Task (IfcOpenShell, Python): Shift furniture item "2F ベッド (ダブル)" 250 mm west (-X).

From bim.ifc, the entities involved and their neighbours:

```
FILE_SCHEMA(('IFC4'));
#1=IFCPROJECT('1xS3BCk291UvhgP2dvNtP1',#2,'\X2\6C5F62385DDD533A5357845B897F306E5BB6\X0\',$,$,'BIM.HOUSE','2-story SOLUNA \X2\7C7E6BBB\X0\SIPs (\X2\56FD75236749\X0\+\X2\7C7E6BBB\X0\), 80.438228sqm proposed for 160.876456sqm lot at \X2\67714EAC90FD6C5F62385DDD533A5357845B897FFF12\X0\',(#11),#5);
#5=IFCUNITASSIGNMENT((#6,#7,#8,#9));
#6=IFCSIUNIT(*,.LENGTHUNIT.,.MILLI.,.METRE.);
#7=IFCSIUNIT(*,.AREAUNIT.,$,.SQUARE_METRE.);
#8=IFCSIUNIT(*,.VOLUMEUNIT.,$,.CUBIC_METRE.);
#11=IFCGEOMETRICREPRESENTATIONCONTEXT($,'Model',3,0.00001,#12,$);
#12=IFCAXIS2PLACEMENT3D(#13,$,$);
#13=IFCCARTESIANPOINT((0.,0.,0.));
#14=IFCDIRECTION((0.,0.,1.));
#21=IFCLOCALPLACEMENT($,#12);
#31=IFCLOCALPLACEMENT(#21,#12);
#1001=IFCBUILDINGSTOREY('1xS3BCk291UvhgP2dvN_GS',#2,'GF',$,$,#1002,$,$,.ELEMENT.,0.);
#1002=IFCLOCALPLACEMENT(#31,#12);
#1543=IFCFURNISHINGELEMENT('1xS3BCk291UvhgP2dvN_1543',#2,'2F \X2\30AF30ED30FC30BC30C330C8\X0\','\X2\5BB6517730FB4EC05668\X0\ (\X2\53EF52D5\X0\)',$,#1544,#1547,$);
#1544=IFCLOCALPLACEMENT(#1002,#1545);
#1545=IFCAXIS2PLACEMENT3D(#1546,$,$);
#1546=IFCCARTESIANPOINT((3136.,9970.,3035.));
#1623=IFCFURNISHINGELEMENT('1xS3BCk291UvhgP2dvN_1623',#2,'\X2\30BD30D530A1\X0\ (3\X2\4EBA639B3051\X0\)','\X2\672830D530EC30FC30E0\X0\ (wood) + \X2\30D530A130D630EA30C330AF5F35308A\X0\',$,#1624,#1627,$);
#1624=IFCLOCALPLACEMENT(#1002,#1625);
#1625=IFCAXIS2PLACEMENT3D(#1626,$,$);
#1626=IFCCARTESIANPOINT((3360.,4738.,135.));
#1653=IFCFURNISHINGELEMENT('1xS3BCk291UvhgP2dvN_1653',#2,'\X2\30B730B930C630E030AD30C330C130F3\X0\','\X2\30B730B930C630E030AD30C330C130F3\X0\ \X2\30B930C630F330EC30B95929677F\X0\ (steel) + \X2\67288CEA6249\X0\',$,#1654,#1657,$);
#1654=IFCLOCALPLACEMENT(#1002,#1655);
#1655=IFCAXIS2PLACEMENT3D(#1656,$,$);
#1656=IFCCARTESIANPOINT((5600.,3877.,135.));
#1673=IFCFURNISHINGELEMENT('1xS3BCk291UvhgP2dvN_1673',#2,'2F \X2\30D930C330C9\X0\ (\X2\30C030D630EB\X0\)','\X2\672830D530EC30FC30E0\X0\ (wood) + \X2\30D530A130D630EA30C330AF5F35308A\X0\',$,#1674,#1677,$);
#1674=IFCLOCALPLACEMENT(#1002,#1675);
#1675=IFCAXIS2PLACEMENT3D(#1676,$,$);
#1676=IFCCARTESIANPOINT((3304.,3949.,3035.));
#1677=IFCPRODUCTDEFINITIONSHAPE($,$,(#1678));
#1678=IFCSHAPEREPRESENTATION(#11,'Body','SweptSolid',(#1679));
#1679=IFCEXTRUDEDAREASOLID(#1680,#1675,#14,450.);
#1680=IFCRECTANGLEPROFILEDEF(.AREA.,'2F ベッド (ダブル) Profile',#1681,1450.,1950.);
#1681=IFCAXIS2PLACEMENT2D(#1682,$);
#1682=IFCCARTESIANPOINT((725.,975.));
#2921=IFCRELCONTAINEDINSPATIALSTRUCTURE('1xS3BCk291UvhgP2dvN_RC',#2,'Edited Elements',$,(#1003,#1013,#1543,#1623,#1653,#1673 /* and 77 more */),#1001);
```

```python
import ifcopenshell
import ifcopenshell.api.geometry
import ifcopenshell.util.placement
import ifcopenshell.util.unit

model = ifcopenshell.open("bim.ifc")
unit_scale = ifcopenshell.util.unit.calculate_unit_scale(model)

item = model.by_guid("1xS3BCk291UvhgP2dvN_1673")
matrix = ifcopenshell.util.placement.get_local_placement(item.ObjectPlacement)
matrix[0, 3] -= 0.25 / unit_scale
ifcopenshell.api.geometry.edit_object_placement(model, product=item, matrix=matrix, is_si=False)

print(ifcopenshell.util.placement.get_local_placement(item.ObjectPlacement).round(3) + 0.0)

model.write("bim_v2.ifc")
```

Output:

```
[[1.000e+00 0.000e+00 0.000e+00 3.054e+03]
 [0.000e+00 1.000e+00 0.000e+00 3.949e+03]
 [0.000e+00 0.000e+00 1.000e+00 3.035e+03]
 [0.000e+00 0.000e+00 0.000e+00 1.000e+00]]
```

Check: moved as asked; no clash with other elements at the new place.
